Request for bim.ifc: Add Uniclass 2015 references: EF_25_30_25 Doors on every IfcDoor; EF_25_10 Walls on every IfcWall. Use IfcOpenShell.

First a look at what the model holds.

```python
import ifcopenshell

model = ifcopenshell.open("bim.ifc")
print(model.schema)
print("classifications:", [c.Name for c in model.by_type("IfcClassification")])
for ifc_class in ("IfcDoor", "IfcRoof", "IfcStair", "IfcWall", "IfcWindow"):
    print(ifc_class, len(model.by_type(ifc_class)))
```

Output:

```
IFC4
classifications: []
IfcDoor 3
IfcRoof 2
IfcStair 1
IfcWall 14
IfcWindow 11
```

```python
import ifcopenshell
import ifcopenshell.api.classification

model = ifcopenshell.open("bim.ifc")

system = ifcopenshell.api.classification.add_classification(model, classification="Uniclass 2015")

codes = {
    "IfcDoor": ("EF_25_30_25", "Doors"),
    "IfcWall": ("EF_25_10", "Walls"),
}
for ifc_class, (code, name) in codes.items():
    products = model.by_type(ifc_class)
    ifcopenshell.api.classification.add_reference(
        model, products=products, classification=system, identification=code, name=name
    )
    print(code, len(products))

model.write("bim_rev.ifc")
```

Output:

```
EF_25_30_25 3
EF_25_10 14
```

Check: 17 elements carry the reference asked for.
